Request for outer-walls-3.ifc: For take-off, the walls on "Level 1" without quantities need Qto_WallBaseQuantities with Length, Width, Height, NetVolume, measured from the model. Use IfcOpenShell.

First a look at what the model holds.

```python
import ifcopenshell
import ifcopenshell.util.element
import ifcopenshell.util.unit

model = ifcopenshell.open("outer-walls-3.ifc")
print(model.schema)
for unit_type in ("LENGTHUNIT", "AREAUNIT", "VOLUMEUNIT"):
    print(unit_type, ifcopenshell.util.unit.calculate_unit_scale(model, unit_type))
storey = next(s for s in model.by_type("IfcBuildingStorey") if s.Name == "Level 1")
walls = [e for e in ifcopenshell.util.element.get_decomposition(storey) if e.is_a("IfcWall")]
for e in sorted(walls, key=lambda e: e.id()):
    print(e.id(), e.is_a(), e.Name, list(ifcopenshell.util.element.get_psets(e, qtos_only=True)), sep=" | ")
```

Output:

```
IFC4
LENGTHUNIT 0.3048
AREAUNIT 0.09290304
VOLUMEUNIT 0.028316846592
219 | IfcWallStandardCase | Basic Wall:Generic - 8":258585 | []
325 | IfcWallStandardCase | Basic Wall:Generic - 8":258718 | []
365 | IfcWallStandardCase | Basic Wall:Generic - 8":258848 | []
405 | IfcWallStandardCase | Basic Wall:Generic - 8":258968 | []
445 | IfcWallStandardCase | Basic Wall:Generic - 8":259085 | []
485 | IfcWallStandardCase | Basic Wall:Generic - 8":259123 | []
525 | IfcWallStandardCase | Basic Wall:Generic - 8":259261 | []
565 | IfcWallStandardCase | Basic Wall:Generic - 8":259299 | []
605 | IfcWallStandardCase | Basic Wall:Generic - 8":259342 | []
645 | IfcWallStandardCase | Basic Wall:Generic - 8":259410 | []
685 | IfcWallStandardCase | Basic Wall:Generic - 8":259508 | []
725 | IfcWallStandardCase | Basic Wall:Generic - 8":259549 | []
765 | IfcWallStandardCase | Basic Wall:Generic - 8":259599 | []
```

```python
import ifcopenshell
import ifcopenshell.api.pset
import ifcopenshell.geom
import ifcopenshell.util.element
import ifcopenshell.util.shape
import ifcopenshell.util.unit

model = ifcopenshell.open("outer-walls-3.ifc")
unit_scale = ifcopenshell.util.unit.calculate_unit_scale(model)
volume_scale = ifcopenshell.util.unit.calculate_unit_scale(model, "VOLUMEUNIT")
settings = ifcopenshell.geom.settings()

storey = next(s for s in model.by_type("IfcBuildingStorey") if s.Name == "Level 1")
walls = [e for e in ifcopenshell.util.element.get_decomposition(storey) if e.is_a("IfcWall")]

for e in sorted(walls, key=lambda e: e.id()):
    if ifcopenshell.util.element.get_psets(e, qtos_only=True, should_inherit=False):
        continue
    # Geometry comes back in metres, in the element's own axes.
    shape = ifcopenshell.geom.create_shape(settings, e)
    values = {
        "Length": ifcopenshell.util.shape.get_x(shape.geometry) / unit_scale,
        "Width": ifcopenshell.util.shape.get_y(shape.geometry) / unit_scale,
        "Height": ifcopenshell.util.shape.get_z(shape.geometry) / unit_scale,
        "NetVolume": ifcopenshell.util.shape.get_volume(shape.geometry) / volume_scale,
    }
    qto = ifcopenshell.api.pset.add_qto(model, product=e, name="Qto_WallBaseQuantities")
    ifcopenshell.api.pset.edit_qto(model, qto=qto, properties=values)
    print(e.id(), {k: round(v, 3) for k, v in values.items()})

model.write("outer-walls-3_v2.ifc")
```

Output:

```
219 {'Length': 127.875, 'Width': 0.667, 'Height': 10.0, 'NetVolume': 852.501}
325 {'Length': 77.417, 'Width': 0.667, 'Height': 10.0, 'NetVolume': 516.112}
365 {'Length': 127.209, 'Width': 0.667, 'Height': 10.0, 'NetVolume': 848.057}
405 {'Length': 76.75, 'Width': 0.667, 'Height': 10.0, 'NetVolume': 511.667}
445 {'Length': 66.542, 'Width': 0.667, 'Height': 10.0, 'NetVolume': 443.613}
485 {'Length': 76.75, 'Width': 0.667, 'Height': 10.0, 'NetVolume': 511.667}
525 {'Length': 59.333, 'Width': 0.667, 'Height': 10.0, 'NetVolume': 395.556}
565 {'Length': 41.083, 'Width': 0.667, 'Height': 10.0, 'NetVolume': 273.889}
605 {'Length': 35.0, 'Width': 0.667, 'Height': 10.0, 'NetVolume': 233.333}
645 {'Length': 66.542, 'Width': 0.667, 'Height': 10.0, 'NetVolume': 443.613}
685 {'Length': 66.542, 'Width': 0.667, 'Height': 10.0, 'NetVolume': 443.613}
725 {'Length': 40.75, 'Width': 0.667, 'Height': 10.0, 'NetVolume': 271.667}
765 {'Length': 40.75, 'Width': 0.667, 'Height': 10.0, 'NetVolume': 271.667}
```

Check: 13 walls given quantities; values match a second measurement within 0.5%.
